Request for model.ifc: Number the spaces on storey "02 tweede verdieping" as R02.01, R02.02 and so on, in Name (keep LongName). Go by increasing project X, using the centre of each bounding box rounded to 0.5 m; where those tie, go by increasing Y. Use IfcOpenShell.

First a look at what the model holds.

```python
import ifcopenshell
import ifcopenshell.util.element
import ifcopenshell.util.placement

model = ifcopenshell.open("model.ifc")
print(model.schema)
storey = next(s for s in model.by_type("IfcBuildingStorey") if s.Name == "02 tweede verdieping")
spaces = [e for e in ifcopenshell.util.element.get_decomposition(storey) if e.is_a("IfcSpace")]
for e in sorted(spaces, key=lambda e: e.id()):
    origin = ifcopenshell.util.placement.get_local_placement(e.ObjectPlacement)[:3, 3]
    print(e.id(), e.Name, e.LongName, origin.round(2) + 0.0, sep=" | ")
```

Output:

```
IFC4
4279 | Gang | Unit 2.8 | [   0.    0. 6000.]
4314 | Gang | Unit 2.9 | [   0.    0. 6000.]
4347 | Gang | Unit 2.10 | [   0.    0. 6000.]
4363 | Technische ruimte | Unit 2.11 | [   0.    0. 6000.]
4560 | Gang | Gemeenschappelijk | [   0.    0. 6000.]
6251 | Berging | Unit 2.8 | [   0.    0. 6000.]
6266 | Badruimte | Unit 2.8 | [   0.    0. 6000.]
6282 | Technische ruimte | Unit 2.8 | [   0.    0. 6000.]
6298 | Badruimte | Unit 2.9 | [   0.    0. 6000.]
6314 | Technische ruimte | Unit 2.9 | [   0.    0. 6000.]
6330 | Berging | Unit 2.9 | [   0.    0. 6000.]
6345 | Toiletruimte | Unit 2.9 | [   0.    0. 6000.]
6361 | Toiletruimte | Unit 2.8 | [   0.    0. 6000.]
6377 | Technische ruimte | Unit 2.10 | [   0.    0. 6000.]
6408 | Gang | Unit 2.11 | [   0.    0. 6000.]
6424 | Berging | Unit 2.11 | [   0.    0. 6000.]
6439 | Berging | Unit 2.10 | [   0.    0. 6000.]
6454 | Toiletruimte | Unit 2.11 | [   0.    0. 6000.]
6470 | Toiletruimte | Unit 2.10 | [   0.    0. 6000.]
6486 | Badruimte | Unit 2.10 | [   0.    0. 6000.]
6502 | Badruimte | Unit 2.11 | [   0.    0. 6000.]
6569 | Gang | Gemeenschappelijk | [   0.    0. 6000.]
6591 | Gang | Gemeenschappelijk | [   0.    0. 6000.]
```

```python
import ifcopenshell
import ifcopenshell.geom
import ifcopenshell.util.element
import ifcopenshell.util.shape

model = ifcopenshell.open("model.ifc")
settings = ifcopenshell.geom.settings()
settings.set("use-world-coords", True)


def centre(element):
    shape = ifcopenshell.geom.create_shape(settings, element)
    return ifcopenshell.util.shape.get_bbox_centroid(shape.geometry)


storey = next(s for s in model.by_type("IfcBuildingStorey") if s.Name == "02 tweede verdieping")
spaces = [e for e in ifcopenshell.util.element.get_decomposition(storey) if e.is_a("IfcSpace")]

# Insertion points can sit at a corner or the storey origin, so sort by the geometry (in metres).
centres = {e: centre(e) for e in spaces}
spaces.sort(key=lambda e: (round(centres[e][0] / 0.5), centres[e][1]))

for i, e in enumerate(spaces, start=1):
    number = f"R02.{i:02d}"
    e.Name = number
    print(e.id(), number)

model.write("model-out.ifc")
```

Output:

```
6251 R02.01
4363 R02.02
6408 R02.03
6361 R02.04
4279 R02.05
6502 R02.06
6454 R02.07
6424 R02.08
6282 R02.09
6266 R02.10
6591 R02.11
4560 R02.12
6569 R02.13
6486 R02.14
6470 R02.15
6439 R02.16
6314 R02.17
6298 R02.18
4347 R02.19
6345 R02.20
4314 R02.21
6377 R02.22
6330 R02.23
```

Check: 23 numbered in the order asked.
